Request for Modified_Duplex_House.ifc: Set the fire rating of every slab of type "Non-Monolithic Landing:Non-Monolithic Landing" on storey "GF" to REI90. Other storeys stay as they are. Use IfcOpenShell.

First a look at what the model holds.

```python
import ifcopenshell
import ifcopenshell.util.element

model = ifcopenshell.open("Modified_Duplex_House.ifc")
print(model.schema)
storey = next(s for s in model.by_type("IfcBuildingStorey") if s.Name == "GF")
slabs = [e for e in ifcopenshell.util.element.get_decomposition(storey) if e.is_a("IfcSlab")]
seen = {}
for e in slabs:
    element_type = ifcopenshell.util.element.get_type(e)
    key = (element_type.Name if element_type != e and element_type else None, ifcopenshell.util.element.get_pset(e, "Pset_SlabCommon", "FireRating"))
    seen[key] = seen.get(key, 0) + 1
for (name, value), count in sorted(seen.items(), key=str):
    print(count, "x", name, "|", value)
```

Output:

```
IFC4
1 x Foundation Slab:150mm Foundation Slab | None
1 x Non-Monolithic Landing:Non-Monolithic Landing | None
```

```python
import ifcopenshell
import ifcopenshell.api.pset
import ifcopenshell.util.element

model = ifcopenshell.open("Modified_Duplex_House.ifc")

storey = next(s for s in model.by_type("IfcBuildingStorey") if s.Name == "GF")
slabs = [e for e in ifcopenshell.util.element.get_decomposition(storey) if e.is_a("IfcSlab")]

count = 0
for e in slabs:
    element_type = ifcopenshell.util.element.get_type(e)
    if element_type in (None, e) or element_type.Name != "Non-Monolithic Landing:Non-Monolithic Landing":
        continue
    # add_pset returns the element's existing set when there is one.
    pset = ifcopenshell.api.pset.add_pset(model, product=e, name="Pset_SlabCommon")
    ifcopenshell.api.pset.edit_pset(model, pset=pset, properties={"FireRating": "REI90"})
    count += 1

print(count, "slabs updated")

model.write("Modified_Duplex_House-out.ifc")
```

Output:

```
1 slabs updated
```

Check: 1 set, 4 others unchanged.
